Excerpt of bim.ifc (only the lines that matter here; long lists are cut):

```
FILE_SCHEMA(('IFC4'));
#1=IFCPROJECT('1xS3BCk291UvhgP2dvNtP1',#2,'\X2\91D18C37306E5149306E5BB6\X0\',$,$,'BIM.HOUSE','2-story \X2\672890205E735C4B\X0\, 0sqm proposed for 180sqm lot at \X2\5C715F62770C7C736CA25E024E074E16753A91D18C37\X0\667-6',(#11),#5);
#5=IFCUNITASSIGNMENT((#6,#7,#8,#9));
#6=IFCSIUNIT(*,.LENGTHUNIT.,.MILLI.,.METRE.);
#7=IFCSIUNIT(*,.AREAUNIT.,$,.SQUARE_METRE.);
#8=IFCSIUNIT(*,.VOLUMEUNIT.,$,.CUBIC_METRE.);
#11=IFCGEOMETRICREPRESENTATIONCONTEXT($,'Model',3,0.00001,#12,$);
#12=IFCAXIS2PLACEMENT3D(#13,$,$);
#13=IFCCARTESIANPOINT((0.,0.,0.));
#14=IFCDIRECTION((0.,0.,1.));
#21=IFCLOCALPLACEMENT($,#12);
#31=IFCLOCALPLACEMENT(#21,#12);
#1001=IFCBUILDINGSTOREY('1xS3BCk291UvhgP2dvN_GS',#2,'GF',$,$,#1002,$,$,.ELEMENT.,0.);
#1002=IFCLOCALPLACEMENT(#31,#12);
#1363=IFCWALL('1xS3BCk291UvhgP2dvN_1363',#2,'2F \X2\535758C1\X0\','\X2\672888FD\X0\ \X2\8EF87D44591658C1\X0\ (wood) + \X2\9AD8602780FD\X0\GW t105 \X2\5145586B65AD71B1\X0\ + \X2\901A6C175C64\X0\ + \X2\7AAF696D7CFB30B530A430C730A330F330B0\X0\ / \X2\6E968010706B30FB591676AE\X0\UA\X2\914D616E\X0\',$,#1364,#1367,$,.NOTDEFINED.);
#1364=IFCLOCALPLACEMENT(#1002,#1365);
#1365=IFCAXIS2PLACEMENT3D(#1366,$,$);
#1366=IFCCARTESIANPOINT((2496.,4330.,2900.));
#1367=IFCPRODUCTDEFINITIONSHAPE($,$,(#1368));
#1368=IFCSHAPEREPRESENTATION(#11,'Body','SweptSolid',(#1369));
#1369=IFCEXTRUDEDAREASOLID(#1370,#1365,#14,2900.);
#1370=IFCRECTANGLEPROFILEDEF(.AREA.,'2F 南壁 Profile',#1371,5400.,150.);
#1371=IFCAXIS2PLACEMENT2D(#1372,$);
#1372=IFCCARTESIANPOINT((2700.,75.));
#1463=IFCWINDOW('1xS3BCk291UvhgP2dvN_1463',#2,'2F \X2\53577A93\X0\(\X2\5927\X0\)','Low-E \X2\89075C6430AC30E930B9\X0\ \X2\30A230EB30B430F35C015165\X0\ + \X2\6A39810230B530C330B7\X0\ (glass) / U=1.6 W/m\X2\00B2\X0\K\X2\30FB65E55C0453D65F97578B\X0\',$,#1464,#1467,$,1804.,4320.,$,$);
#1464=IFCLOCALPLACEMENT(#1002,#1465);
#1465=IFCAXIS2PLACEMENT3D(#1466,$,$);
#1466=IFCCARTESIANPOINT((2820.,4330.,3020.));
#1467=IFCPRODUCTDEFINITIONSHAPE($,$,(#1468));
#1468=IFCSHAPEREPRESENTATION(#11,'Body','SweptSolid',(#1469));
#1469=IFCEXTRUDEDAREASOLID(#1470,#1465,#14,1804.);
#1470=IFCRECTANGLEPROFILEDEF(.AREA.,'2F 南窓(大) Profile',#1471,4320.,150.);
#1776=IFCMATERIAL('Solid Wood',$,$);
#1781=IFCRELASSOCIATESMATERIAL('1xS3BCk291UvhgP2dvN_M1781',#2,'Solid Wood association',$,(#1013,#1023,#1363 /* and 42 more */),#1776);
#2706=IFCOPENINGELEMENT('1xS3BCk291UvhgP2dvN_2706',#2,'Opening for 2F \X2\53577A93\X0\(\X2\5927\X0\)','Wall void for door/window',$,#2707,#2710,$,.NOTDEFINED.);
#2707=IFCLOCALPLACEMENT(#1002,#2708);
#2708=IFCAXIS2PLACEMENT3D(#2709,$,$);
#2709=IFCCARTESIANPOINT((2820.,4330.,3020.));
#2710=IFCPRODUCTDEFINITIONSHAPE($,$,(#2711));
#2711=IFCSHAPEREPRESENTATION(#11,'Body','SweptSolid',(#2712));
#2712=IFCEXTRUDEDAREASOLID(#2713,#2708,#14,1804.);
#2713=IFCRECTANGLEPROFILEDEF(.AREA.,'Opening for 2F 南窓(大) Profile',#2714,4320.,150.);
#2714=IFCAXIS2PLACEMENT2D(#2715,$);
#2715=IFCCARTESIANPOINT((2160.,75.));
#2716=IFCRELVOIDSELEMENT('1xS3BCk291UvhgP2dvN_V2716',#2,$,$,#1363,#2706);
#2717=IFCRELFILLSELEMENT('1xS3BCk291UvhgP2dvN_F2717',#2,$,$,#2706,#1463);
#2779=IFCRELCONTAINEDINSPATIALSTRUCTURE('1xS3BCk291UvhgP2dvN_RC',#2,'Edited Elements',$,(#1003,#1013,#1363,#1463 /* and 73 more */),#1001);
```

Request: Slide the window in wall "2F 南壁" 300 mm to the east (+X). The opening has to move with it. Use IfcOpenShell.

```python
import ifcopenshell
import ifcopenshell.api.geometry
import ifcopenshell.util.placement

model = ifcopenshell.open("bim.ifc")

window = model.by_guid("1xS3BCk291UvhgP2dvN_1463")
opening = window.FillsVoids[0].RelatingOpeningElement
wall = opening.VoidsElements[0].RelatingBuildingElement

wall_matrix = ifcopenshell.util.placement.get_local_placement(wall.ObjectPlacement)
shift = wall_matrix[:3, 0] * 300.0
before = ifcopenshell.util.placement.get_local_placement(window.ObjectPlacement)[:3, 3].copy()

# The window is not placed relative to its opening, so move both.
for product in (opening, window):
    matrix = ifcopenshell.util.placement.get_local_placement(product.ObjectPlacement)
    matrix[:3, 3] += shift
    ifcopenshell.api.geometry.edit_object_placement(model, product=product, matrix=matrix, is_si=False)

after = ifcopenshell.util.placement.get_local_placement(window.ObjectPlacement)[:3, 3]
print("window moved by", (after - before).round(3) + 0.0)

model.write("bim_rev.ifc")
```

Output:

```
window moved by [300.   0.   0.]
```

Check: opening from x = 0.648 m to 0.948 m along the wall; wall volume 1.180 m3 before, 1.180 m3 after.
